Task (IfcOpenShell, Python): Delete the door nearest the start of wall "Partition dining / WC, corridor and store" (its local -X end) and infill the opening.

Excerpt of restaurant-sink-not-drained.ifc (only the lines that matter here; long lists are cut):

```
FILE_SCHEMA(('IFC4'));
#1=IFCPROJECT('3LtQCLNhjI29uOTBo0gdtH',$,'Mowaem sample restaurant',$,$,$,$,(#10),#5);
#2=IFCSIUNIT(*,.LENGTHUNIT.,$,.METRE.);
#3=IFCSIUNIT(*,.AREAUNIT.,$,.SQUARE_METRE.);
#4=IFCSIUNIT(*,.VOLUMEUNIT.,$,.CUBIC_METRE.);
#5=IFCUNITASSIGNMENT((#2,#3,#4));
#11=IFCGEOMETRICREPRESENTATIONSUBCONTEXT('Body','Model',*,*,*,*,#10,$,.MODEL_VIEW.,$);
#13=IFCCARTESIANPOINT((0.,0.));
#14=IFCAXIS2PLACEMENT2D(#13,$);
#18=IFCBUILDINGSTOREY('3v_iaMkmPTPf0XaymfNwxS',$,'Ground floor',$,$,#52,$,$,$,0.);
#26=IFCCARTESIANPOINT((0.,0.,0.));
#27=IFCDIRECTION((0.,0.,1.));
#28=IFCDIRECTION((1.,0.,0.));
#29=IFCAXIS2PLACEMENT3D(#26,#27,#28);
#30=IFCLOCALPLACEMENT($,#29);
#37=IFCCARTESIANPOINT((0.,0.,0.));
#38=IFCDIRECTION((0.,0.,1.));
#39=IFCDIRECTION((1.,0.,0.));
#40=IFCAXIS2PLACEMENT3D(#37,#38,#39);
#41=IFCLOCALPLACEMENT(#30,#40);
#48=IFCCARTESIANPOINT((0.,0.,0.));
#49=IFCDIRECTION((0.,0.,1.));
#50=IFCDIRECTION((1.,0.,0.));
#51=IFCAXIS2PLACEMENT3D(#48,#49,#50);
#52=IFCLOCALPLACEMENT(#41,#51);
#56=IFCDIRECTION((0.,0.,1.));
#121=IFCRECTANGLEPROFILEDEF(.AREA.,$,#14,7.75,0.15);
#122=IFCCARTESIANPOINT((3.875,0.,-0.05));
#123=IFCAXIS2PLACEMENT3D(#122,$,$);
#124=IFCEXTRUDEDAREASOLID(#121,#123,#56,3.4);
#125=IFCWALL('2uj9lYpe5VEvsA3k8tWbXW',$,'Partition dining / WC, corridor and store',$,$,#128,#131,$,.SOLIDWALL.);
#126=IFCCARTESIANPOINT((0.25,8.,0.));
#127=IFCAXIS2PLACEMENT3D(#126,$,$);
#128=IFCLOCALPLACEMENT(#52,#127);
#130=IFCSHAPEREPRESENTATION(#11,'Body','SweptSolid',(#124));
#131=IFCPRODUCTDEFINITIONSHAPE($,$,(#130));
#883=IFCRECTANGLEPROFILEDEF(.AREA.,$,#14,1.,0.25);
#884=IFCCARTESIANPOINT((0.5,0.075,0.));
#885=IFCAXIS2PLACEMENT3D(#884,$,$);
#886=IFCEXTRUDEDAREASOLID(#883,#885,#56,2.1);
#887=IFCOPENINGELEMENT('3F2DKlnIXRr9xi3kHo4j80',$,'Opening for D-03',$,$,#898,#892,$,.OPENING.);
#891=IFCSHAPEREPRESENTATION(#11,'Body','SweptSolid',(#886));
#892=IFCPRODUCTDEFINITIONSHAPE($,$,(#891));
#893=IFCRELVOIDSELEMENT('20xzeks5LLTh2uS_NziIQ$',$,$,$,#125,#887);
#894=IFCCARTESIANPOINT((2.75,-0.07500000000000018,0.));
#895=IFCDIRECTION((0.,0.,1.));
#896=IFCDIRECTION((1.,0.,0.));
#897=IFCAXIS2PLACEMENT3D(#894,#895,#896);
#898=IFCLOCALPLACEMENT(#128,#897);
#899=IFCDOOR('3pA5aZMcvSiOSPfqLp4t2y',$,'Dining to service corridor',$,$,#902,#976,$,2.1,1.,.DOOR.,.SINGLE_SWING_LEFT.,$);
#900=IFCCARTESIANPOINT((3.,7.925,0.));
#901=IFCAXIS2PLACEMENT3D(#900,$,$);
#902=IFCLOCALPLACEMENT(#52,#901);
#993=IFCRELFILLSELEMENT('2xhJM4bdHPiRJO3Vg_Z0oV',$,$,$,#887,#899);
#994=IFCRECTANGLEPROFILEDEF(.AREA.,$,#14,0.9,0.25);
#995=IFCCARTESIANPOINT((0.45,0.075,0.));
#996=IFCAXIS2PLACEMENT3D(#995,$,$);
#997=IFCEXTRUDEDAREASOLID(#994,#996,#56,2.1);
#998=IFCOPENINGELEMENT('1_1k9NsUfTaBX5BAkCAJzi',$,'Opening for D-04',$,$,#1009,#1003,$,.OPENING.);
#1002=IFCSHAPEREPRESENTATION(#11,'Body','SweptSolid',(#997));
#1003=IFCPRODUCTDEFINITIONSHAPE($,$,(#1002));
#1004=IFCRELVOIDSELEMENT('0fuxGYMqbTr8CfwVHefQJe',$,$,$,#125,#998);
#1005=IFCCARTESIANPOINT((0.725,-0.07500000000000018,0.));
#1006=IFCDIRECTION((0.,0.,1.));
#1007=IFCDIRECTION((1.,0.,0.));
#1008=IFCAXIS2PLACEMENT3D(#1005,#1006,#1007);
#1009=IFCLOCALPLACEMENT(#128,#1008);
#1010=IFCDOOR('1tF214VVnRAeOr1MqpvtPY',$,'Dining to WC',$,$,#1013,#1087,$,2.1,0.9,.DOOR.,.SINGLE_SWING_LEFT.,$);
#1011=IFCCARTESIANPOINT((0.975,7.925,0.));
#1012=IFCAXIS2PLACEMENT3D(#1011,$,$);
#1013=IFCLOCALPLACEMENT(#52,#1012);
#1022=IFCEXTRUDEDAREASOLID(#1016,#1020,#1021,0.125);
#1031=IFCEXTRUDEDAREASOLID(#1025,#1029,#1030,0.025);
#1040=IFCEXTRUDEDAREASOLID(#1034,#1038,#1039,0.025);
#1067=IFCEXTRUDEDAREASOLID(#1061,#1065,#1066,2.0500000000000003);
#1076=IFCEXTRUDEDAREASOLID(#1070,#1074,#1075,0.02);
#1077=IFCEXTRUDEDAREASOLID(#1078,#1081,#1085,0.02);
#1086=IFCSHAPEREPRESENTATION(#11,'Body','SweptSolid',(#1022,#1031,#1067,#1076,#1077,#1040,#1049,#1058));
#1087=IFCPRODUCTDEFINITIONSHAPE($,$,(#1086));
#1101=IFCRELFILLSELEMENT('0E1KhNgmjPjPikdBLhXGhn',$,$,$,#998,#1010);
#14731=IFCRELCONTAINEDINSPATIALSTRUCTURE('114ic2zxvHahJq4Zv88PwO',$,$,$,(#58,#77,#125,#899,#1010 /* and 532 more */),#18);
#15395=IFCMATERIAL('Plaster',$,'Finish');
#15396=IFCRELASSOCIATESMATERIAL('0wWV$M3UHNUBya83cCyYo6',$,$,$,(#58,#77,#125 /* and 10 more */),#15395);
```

```python
import ifcopenshell
import ifcopenshell.api.feature
import ifcopenshell.api.root
import ifcopenshell.geom
import ifcopenshell.util.shape

model = ifcopenshell.open("restaurant-sink-not-drained.ifc")
settings = ifcopenshell.geom.settings()


def volume(element):
    """Net volume in cubic metres, openings subtracted."""
    shape = ifcopenshell.geom.create_shape(settings, element)
    return ifcopenshell.util.shape.get_volume(shape.geometry)


door = model.by_guid("1tF214VVnRAeOr1MqpvtPY")
opening = door.FillsVoids[0].RelatingOpeningElement
wall = opening.VoidsElements[0].RelatingBuildingElement
before = volume(wall)

ifcopenshell.api.root.remove_product(model, product=door)
ifcopenshell.api.feature.remove_feature(model, feature=opening)

after = volume(wall)

print(f"wall volume {before:.3f} -> {after:.3f} m3")

model.write("restaurant-sink-not-drained_rev.ifc")
```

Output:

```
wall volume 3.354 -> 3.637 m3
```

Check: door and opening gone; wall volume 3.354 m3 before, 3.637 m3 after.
